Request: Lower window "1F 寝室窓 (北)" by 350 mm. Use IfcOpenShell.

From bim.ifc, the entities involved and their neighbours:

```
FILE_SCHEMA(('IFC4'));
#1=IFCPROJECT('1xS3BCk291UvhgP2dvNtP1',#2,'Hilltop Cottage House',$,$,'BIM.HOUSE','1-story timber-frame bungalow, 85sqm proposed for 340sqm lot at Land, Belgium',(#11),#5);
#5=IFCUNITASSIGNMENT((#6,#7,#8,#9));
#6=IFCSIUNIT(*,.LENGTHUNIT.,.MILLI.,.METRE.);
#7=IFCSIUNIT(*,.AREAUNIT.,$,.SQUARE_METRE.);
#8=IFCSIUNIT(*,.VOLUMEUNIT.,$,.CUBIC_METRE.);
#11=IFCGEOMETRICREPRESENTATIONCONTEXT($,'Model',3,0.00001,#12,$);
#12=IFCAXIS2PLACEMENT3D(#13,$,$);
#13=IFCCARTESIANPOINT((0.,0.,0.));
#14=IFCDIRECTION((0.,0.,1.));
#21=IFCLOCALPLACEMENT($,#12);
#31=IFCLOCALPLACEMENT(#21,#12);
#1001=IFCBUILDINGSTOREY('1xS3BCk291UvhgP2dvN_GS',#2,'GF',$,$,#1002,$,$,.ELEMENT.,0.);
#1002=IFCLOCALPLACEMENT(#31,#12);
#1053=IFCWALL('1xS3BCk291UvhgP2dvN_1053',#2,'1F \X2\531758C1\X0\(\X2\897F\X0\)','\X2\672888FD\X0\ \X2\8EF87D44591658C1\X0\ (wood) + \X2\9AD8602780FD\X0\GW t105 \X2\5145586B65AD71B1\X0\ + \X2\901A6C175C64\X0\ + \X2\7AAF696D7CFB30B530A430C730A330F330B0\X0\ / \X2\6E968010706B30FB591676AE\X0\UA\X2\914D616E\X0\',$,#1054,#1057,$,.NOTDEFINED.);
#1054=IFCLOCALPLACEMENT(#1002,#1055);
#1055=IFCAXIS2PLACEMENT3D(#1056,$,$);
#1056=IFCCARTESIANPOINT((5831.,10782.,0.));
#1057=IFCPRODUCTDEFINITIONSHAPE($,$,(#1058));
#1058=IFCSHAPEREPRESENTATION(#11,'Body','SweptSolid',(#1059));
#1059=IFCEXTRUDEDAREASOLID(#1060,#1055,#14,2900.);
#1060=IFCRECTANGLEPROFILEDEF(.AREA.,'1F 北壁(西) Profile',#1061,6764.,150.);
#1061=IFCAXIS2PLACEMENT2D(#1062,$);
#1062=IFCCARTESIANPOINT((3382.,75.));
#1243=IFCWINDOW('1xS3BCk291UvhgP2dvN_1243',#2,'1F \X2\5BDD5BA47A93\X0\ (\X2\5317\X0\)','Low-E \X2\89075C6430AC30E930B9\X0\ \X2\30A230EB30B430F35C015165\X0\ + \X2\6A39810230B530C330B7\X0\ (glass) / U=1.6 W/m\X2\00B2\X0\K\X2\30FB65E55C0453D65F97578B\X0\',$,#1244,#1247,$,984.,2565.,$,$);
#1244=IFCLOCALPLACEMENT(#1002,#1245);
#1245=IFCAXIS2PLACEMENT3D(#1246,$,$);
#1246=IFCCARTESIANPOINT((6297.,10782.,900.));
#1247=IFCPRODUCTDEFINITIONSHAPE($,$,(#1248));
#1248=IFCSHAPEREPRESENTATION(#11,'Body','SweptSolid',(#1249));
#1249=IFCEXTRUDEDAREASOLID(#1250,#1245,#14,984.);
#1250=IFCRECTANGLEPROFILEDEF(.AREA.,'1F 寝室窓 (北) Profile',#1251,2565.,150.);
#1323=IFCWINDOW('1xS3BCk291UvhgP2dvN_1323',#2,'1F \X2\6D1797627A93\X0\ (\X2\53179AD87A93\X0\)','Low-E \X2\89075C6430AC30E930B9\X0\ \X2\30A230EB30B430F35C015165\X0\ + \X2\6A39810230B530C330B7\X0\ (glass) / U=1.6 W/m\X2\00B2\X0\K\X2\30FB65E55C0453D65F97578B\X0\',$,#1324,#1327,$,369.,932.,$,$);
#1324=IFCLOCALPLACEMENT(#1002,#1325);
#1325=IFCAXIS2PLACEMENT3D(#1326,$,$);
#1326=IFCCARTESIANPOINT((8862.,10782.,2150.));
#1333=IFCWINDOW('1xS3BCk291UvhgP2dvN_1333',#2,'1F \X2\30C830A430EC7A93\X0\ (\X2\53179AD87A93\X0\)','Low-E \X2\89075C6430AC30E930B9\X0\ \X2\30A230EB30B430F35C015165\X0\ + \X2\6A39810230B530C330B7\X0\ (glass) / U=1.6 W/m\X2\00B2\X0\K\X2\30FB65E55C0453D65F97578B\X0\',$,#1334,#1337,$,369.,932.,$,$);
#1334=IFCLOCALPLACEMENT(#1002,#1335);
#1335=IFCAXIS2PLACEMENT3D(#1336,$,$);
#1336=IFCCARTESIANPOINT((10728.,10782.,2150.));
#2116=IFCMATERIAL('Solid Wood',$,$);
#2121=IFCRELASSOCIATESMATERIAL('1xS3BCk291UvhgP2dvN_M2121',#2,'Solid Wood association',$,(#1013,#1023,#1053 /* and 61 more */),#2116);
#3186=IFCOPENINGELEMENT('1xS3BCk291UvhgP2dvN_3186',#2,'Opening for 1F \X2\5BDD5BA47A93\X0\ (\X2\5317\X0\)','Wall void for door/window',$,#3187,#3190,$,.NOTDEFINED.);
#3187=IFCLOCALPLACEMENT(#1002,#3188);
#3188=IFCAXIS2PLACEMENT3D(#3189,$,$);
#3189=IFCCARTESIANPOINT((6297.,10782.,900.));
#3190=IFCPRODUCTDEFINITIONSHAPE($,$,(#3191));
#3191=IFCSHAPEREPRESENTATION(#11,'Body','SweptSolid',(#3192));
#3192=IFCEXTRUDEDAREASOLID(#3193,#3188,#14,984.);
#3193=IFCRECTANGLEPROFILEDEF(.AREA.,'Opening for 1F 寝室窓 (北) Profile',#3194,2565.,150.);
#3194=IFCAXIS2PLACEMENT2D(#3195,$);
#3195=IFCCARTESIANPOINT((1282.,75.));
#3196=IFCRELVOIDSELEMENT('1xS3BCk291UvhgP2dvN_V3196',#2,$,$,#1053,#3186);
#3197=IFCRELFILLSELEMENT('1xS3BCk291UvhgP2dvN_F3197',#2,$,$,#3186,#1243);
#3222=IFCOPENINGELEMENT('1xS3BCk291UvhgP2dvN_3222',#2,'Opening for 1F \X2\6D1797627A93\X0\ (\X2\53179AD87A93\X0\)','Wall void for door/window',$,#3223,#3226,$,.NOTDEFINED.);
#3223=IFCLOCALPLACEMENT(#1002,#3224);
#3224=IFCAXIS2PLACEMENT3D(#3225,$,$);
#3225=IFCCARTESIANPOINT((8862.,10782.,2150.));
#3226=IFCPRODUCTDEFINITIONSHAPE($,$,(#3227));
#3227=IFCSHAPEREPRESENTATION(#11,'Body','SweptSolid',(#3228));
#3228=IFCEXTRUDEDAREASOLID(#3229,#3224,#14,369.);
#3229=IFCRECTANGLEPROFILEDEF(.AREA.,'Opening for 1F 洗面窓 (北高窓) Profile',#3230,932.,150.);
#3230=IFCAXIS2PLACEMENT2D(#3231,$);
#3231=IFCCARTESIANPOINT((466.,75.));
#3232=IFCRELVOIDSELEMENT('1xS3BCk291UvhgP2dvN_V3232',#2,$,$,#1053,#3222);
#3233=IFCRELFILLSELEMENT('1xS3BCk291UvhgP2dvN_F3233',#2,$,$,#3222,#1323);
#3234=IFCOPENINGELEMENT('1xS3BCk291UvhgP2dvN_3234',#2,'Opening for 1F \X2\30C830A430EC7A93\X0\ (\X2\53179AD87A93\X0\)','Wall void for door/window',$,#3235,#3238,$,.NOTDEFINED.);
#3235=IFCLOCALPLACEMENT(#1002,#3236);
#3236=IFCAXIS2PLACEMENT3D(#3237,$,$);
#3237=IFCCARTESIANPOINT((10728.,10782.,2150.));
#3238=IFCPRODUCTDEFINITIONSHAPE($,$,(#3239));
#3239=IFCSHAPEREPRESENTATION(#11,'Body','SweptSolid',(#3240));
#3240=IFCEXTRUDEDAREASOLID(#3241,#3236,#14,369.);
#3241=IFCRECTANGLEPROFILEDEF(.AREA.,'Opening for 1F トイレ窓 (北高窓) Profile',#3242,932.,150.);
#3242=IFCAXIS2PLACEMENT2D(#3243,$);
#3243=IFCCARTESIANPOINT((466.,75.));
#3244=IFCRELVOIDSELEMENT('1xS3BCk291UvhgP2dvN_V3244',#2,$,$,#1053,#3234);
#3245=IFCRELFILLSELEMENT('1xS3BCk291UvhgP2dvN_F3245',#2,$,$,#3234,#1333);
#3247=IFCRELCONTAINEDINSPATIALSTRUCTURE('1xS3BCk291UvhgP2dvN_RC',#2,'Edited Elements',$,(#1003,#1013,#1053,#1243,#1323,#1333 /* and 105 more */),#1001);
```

```python
import numpy as np
import ifcopenshell
import ifcopenshell.api.geometry
import ifcopenshell.util.placement
import ifcopenshell.util.unit

model = ifcopenshell.open("bim.ifc")
unit_scale = ifcopenshell.util.unit.calculate_unit_scale(model)

window = model.by_guid("1xS3BCk291UvhgP2dvN_1243")
opening = window.FillsVoids[0].RelatingOpeningElement
dz = -0.35 / unit_scale

shift = np.array([0.0, 0.0, dz])
# The window is not placed relative to its opening, so move both.
for product in (opening, window):
    matrix = ifcopenshell.util.placement.get_local_placement(product.ObjectPlacement)
    matrix[:3, 3] += shift
    ifcopenshell.api.geometry.edit_object_placement(model, product=product, matrix=matrix, is_si=False)

print(f"moved by {dz * unit_scale:+.3f} m")

model.write("bim_rev.ifc")
```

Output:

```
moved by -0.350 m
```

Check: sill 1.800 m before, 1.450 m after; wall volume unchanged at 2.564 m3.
